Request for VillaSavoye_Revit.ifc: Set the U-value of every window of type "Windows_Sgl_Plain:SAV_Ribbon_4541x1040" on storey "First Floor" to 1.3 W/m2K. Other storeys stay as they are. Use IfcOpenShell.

First a look at what the model holds.

```python
import ifcopenshell
import ifcopenshell.util.element

model = ifcopenshell.open("VillaSavoye_Revit.ifc")
print(model.schema)
storey = next(s for s in model.by_type("IfcBuildingStorey") if s.Name == "First Floor")
windows = [e for e in ifcopenshell.util.element.get_decomposition(storey) if e.is_a("IfcWindow")]
seen = {}
for e in windows:
    element_type = ifcopenshell.util.element.get_type(e)
    key = (element_type.Name if element_type != e and element_type else None, ifcopenshell.util.element.get_pset(e, "Pset_WindowCommon", "ThermalTransmittance"))
    seen[key] = seen.get(key, 0) + 1
for (name, value), count in sorted(seen.items(), key=str):
    print(count, "x", name, "|", value)
```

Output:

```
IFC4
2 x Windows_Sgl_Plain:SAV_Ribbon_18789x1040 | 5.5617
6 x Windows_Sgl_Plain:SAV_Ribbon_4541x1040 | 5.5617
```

```python
import ifcopenshell
import ifcopenshell.api.pset
import ifcopenshell.util.element

model = ifcopenshell.open("VillaSavoye_Revit.ifc")

storey = next(s for s in model.by_type("IfcBuildingStorey") if s.Name == "First Floor")
windows = [e for e in ifcopenshell.util.element.get_decomposition(storey) if e.is_a("IfcWindow")]

count = 0
for e in windows:
    element_type = ifcopenshell.util.element.get_type(e)
    if element_type in (None, e) or element_type.Name != "Windows_Sgl_Plain:SAV_Ribbon_4541x1040":
        continue
    # add_pset returns the element's existing set when there is one.
    pset = ifcopenshell.api.pset.add_pset(model, product=e, name="Pset_WindowCommon")
    ifcopenshell.api.pset.edit_pset(model, pset=pset, properties={"ThermalTransmittance": 1.3})
    count += 1

print(count, "windows updated")

model.write("VillaSavoye_Revit-out.ifc")
```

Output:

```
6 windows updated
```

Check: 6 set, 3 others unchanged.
